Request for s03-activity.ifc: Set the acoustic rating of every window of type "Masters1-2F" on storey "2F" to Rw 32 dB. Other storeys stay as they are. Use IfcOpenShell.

First a look at what the model holds.

```python
import ifcopenshell
import ifcopenshell.util.element

model = ifcopenshell.open("s03-activity.ifc")
print(model.schema)
storey = next(s for s in model.by_type("IfcBuildingStorey") if s.Name == "2F")
windows = [e for e in ifcopenshell.util.element.get_decomposition(storey) if e.is_a("IfcWindow")]
seen = {}
for e in windows:
    element_type = ifcopenshell.util.element.get_type(e)
    key = (element_type.Name if element_type != e and element_type else None, ifcopenshell.util.element.get_pset(e, "Pset_WindowCommon", "AcousticRating"))
    seen[key] = seen.get(key, 0) + 1
for (name, value), count in sorted(seen.items(), key=str):
    print(count, "x", name, "|", value)
```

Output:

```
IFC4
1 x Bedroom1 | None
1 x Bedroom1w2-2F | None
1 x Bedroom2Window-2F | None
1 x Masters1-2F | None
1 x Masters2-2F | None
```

```python
import ifcopenshell
import ifcopenshell.api.pset
import ifcopenshell.util.element

model = ifcopenshell.open("s03-activity.ifc")

storey = next(s for s in model.by_type("IfcBuildingStorey") if s.Name == "2F")
windows = [e for e in ifcopenshell.util.element.get_decomposition(storey) if e.is_a("IfcWindow")]

count = 0
for e in windows:
    element_type = ifcopenshell.util.element.get_type(e)
    if element_type in (None, e) or element_type.Name != "Masters1-2F":
        continue
    # add_pset returns the element's existing set when there is one.
    pset = ifcopenshell.api.pset.add_pset(model, product=e, name="Pset_WindowCommon")
    ifcopenshell.api.pset.edit_pset(model, pset=pset, properties={"AcousticRating": "Rw 32 dB"})
    count += 1

print(count, "windows updated")

model.write("s03-activity_updated.ifc")
```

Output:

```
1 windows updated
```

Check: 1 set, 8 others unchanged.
